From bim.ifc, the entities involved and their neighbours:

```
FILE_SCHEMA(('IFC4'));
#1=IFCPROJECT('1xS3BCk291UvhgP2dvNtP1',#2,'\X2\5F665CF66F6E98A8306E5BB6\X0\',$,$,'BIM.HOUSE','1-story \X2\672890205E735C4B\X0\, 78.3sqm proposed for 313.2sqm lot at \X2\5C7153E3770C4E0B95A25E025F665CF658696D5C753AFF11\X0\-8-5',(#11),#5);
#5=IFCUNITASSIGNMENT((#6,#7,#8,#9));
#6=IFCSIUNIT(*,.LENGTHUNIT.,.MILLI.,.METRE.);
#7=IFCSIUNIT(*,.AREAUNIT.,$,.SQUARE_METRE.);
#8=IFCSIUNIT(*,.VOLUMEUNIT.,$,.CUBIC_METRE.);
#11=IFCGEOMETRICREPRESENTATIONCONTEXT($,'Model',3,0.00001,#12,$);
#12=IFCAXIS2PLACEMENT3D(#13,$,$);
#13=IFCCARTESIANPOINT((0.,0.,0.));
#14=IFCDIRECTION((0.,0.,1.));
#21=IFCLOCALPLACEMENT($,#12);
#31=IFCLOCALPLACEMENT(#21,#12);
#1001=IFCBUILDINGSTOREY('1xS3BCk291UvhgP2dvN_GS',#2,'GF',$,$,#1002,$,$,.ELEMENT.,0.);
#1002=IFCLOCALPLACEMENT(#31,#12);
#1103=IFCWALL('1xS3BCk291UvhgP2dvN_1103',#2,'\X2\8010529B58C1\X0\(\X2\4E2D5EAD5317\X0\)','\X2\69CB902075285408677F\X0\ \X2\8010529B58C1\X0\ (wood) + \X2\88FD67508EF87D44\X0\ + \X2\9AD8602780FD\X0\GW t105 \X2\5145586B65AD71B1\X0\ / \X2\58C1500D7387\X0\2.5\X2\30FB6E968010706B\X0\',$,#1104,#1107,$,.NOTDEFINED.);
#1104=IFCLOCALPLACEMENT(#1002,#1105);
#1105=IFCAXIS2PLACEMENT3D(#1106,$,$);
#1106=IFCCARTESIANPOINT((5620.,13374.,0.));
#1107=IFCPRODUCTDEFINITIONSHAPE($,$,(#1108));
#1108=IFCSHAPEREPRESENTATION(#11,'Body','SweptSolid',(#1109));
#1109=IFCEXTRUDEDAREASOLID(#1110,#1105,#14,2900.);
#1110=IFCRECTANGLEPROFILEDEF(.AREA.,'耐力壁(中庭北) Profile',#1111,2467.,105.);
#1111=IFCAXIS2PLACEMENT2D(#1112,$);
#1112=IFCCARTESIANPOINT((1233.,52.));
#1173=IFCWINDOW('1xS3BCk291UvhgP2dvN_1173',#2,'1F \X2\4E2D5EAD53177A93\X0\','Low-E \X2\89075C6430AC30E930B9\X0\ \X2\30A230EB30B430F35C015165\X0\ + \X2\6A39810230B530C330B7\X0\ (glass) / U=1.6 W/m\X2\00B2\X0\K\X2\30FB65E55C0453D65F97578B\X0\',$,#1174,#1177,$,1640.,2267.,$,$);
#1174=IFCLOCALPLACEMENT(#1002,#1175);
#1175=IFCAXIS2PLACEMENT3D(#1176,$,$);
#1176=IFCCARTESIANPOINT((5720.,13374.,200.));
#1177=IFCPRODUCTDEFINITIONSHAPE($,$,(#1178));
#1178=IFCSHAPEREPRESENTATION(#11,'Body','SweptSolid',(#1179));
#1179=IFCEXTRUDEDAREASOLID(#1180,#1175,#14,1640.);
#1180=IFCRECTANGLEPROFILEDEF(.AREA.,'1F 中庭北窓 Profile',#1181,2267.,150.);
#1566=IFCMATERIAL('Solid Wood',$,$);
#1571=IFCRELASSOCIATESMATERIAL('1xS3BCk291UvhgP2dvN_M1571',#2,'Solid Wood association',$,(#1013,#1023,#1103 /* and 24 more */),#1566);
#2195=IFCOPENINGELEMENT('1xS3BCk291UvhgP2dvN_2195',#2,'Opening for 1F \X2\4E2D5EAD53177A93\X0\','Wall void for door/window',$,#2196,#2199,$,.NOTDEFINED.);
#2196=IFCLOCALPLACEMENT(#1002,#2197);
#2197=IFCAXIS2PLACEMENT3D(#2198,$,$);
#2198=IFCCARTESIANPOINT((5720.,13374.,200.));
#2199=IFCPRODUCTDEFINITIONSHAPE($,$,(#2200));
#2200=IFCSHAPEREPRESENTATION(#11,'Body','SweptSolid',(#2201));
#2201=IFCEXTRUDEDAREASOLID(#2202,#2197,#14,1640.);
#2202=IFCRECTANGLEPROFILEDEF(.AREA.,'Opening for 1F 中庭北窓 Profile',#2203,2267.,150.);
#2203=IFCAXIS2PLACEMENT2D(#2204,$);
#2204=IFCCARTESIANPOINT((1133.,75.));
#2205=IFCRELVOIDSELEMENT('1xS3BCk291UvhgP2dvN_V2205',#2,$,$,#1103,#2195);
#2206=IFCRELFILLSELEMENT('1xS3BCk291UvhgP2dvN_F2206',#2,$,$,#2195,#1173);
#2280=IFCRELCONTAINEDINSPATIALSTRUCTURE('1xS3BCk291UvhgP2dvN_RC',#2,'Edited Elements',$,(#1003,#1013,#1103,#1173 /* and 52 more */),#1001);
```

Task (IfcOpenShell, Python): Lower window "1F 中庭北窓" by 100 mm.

```python
import numpy as np
import ifcopenshell
import ifcopenshell.api.geometry
import ifcopenshell.util.placement
import ifcopenshell.util.unit

model = ifcopenshell.open("bim.ifc")
unit_scale = ifcopenshell.util.unit.calculate_unit_scale(model)

window = model.by_guid("1xS3BCk291UvhgP2dvN_1173")
opening = window.FillsVoids[0].RelatingOpeningElement
dz = -100.0

shift = np.array([0.0, 0.0, dz])
# The window is not placed relative to its opening, so move both.
for product in (opening, window):
    matrix = ifcopenshell.util.placement.get_local_placement(product.ObjectPlacement)
    matrix[:3, 3] += shift
    ifcopenshell.api.geometry.edit_object_placement(model, product=product, matrix=matrix, is_si=False)

print(f"moved by {dz * unit_scale:+.3f} m")

model.write("bim_rev.ifc")
```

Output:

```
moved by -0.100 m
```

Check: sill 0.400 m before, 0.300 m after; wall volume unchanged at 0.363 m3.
